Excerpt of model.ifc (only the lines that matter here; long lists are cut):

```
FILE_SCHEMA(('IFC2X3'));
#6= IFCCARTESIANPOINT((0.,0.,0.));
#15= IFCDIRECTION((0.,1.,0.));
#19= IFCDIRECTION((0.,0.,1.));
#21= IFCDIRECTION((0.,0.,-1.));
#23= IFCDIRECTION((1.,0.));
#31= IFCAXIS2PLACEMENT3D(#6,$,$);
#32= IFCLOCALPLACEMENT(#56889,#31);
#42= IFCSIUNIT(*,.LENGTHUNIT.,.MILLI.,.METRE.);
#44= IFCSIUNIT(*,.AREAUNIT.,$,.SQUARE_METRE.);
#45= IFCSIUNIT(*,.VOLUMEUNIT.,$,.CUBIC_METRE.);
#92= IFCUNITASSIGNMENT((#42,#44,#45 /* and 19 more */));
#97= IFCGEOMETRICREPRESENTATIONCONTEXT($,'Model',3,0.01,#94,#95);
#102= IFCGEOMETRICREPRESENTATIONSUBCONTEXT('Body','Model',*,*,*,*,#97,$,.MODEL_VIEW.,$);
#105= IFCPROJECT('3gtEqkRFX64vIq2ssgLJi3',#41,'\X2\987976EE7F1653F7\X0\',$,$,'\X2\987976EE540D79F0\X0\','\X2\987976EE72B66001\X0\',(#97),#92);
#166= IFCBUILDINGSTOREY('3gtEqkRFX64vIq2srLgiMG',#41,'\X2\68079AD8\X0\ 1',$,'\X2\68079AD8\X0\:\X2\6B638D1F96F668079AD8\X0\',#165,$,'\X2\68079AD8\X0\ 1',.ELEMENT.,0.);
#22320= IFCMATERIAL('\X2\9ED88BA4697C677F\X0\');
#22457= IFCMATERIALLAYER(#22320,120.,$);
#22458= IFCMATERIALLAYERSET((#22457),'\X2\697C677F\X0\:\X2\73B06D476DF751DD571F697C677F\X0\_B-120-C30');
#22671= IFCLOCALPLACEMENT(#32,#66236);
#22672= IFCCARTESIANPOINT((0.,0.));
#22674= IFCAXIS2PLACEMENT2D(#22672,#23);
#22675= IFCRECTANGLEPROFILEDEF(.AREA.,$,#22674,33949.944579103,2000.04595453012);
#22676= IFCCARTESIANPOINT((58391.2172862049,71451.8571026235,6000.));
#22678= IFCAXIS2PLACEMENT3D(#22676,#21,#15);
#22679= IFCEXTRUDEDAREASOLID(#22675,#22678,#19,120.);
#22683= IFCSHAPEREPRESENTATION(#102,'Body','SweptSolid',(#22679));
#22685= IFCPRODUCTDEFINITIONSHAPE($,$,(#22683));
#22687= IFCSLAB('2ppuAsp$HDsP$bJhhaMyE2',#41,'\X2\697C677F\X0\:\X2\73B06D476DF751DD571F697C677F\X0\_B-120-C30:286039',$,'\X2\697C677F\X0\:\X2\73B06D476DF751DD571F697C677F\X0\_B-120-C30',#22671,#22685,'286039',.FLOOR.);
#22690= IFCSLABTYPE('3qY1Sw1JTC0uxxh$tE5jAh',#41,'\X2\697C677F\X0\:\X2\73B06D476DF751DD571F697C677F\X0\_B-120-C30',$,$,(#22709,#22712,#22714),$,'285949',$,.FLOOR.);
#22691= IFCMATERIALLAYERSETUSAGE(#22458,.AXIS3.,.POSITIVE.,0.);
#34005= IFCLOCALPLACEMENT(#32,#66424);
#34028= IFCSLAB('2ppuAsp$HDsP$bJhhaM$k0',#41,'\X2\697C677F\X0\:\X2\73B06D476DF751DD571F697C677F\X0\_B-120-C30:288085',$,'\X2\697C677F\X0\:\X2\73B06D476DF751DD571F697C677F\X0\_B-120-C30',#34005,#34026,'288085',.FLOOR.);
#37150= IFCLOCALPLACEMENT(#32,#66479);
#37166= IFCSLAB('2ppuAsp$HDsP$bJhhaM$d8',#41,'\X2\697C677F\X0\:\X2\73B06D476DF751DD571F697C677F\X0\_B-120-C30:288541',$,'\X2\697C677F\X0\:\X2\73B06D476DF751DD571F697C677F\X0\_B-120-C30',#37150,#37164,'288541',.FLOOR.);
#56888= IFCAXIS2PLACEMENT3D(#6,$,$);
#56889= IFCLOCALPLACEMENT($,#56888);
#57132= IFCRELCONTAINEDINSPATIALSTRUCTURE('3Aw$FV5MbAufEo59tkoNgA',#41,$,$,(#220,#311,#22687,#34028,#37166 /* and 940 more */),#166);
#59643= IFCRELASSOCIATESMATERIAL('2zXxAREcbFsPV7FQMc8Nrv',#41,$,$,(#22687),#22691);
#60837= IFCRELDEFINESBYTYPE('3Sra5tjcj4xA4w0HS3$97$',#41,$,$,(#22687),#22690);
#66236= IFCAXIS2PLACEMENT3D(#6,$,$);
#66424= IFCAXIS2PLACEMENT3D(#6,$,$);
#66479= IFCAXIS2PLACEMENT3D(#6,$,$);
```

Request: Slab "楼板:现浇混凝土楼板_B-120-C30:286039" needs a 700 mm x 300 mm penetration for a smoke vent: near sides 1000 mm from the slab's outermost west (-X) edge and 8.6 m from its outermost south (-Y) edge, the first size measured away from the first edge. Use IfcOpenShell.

```python
import numpy as np
import ifcopenshell
import ifcopenshell.api.feature
import ifcopenshell.api.geometry
import ifcopenshell.api.root
import ifcopenshell.geom
import ifcopenshell.util.placement
import ifcopenshell.util.representation
import ifcopenshell.util.shape
import ifcopenshell.util.unit

model = ifcopenshell.open("model.ifc")
unit_scale = ifcopenshell.util.unit.calculate_unit_scale(model)
settings = ifcopenshell.geom.settings()


def volume(element):
    """Net volume in cubic metres, openings subtracted."""
    shape = ifcopenshell.geom.create_shape(settings, element)
    return ifcopenshell.util.shape.get_volume(shape.geometry)


slab = model.by_id(22687)
before = volume(slab)

# Extent in the slab's own axes, in metres. The edges named are its -X and -Y sides.
slab_shape = ifcopenshell.geom.create_shape(settings, slab)
vertices = ifcopenshell.util.shape.get_vertices(slab_shape.geometry)
x_min, y_min, bottom = vertices.min(axis=0)
top = vertices[:, 2].max()

opening = ifcopenshell.api.root.create_entity(model, ifc_class="IfcOpeningElement", name="Smoke vent opening")
context = ifcopenshell.util.representation.get_context(model, "Model", "Body", "MODEL_VIEW")
width, depth = 0.7, 0.3
outline = [(0.0, 0.0), (width, 0.0), (width, depth), (0.0, depth), (0.0, 0.0)]
# Overshoot both faces by 50 mm so the cut is clean.
shape = ifcopenshell.api.geometry.add_slab_representation(
    model, context=context, depth=top - bottom + 0.1, polyline=outline
)
ifcopenshell.api.geometry.assign_representation(model, product=opening, representation=shape)

matrix = ifcopenshell.util.placement.get_local_placement(slab.ObjectPlacement)
matrix[:, 3] = matrix @ np.append(np.array([x_min + 1, y_min + 8.6, bottom - 0.05]) / unit_scale, 1.0)
ifcopenshell.api.geometry.edit_object_placement(model, product=opening, matrix=matrix, is_si=False)
ifcopenshell.api.feature.add_feature(model, feature=opening, element=slab)

after = volume(slab)

print(f"slab volume {before:.3f} -> {after:.3f} m3")

model.write("model-out.ifc")
```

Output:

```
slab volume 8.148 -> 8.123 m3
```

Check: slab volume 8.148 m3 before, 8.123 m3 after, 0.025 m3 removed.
